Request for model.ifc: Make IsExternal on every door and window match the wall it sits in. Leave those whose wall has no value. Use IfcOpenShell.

First a look at what the model holds.

```python
import ifcopenshell
import ifcopenshell.util.element

model = ifcopenshell.open("model.ifc")
print(model.schema)
seen = {}
for e in model.by_type("IfcDoor") + model.by_type("IfcWindow"):
    if not e.FillsVoids:
        continue
    host = e.FillsVoids[0].RelatingOpeningElement.VoidsElements[0].RelatingBuildingElement
    own = ifcopenshell.util.element.get_pset(e, f"Pset_{e.is_a()[3:].removesuffix('StandardCase')}Common", "IsExternal")
    wall = ifcopenshell.util.element.get_pset(host, "Pset_WallCommon", "IsExternal")
    seen[e.is_a(), own, wall] = seen.get((e.is_a(), own, wall), 0) + 1
for (cls, own, wall), count in sorted(seen.items(), key=str):
    print(count, cls, "IsExternal:", own, "| host wall:", wall)
```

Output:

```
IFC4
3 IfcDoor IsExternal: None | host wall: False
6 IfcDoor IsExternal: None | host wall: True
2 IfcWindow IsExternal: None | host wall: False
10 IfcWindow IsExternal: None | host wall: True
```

```python
import ifcopenshell
import ifcopenshell.api.pset
import ifcopenshell.util.element

model = ifcopenshell.open("model.ifc")

count = 0
for ifc_class, pset_name in (("IfcDoor", "Pset_DoorCommon"), ("IfcWindow", "Pset_WindowCommon")):
    for e in model.by_type(ifc_class):
        if not e.FillsVoids:
            continue
        host = e.FillsVoids[0].RelatingOpeningElement.VoidsElements[0].RelatingBuildingElement
        external = ifcopenshell.util.element.get_pset(host, "Pset_WallCommon", "IsExternal")
        if external is None or ifcopenshell.util.element.get_pset(e, pset_name, "IsExternal") == external:
            continue
        pset = ifcopenshell.api.pset.add_pset(model, product=e, name=pset_name)
        ifcopenshell.api.pset.edit_pset(model, pset=pset, properties={"IsExternal": external})
        count += 1

print(count, "updated")

model.write("model_rev.ifc")
```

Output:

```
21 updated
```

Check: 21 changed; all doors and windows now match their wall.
